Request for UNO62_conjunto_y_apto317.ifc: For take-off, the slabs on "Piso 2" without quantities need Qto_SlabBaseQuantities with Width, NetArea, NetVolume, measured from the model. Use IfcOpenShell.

First a look at what the model holds.

```python
import ifcopenshell
import ifcopenshell.util.element
import ifcopenshell.util.unit

model = ifcopenshell.open("UNO62_conjunto_y_apto317.ifc")
print(model.schema)
for unit_type in ("LENGTHUNIT", "AREAUNIT", "VOLUMEUNIT"):
    print(unit_type, ifcopenshell.util.unit.calculate_unit_scale(model, unit_type))
storey = next(s for s in model.by_type("IfcBuildingStorey") if s.Name == "Piso 2")
slabs = [e for e in ifcopenshell.util.element.get_decomposition(storey) if e.is_a("IfcSlab")]
for e in sorted(slabs, key=lambda e: e.id()):
    print(e.id(), e.is_a(), e.Name, list(ifcopenshell.util.element.get_psets(e, qtos_only=True)), sep=" | ")
```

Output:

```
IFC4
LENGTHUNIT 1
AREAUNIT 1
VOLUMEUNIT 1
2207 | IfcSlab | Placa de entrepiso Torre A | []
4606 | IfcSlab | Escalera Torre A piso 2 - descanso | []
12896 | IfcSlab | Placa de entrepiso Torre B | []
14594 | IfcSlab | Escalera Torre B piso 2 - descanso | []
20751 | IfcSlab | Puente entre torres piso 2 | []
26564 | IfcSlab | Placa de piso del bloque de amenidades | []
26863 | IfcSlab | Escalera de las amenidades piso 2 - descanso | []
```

```python
import ifcopenshell
import ifcopenshell.api.pset
import ifcopenshell.geom
import ifcopenshell.util.element
import ifcopenshell.util.shape
import ifcopenshell.util.unit

model = ifcopenshell.open("UNO62_conjunto_y_apto317.ifc")
unit_scale = ifcopenshell.util.unit.calculate_unit_scale(model)
area_scale = ifcopenshell.util.unit.calculate_unit_scale(model, "AREAUNIT")
volume_scale = ifcopenshell.util.unit.calculate_unit_scale(model, "VOLUMEUNIT")
settings = ifcopenshell.geom.settings()

storey = next(s for s in model.by_type("IfcBuildingStorey") if s.Name == "Piso 2")
slabs = [e for e in ifcopenshell.util.element.get_decomposition(storey) if e.is_a("IfcSlab")]

for e in sorted(slabs, key=lambda e: e.id()):
    if ifcopenshell.util.element.get_psets(e, qtos_only=True, should_inherit=False):
        continue
    # Geometry comes back in metres, in the element's own axes.
    shape = ifcopenshell.geom.create_shape(settings, e)
    values = {
        "Width": ifcopenshell.util.shape.get_z(shape.geometry) / unit_scale,
        "NetArea": ifcopenshell.util.shape.get_footprint_area(shape.geometry) / area_scale,
        "NetVolume": ifcopenshell.util.shape.get_volume(shape.geometry) / volume_scale,
    }
    qto = ifcopenshell.api.pset.add_qto(model, product=e, name="Qto_SlabBaseQuantities")
    ifcopenshell.api.pset.edit_qto(model, qto=qto, properties=values)
    print(e.id(), {k: round(v, 3) for k, v in values.items()})

model.write("UNO62_conjunto_y_apto317-out.ifc")
```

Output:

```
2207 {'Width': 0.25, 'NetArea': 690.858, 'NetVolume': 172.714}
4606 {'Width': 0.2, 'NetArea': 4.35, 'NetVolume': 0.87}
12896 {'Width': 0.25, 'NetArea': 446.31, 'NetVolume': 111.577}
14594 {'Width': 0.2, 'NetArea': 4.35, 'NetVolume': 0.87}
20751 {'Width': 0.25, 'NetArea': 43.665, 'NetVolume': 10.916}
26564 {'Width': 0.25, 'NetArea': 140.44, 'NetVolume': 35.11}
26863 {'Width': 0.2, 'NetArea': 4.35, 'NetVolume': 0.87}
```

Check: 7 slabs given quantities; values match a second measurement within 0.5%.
